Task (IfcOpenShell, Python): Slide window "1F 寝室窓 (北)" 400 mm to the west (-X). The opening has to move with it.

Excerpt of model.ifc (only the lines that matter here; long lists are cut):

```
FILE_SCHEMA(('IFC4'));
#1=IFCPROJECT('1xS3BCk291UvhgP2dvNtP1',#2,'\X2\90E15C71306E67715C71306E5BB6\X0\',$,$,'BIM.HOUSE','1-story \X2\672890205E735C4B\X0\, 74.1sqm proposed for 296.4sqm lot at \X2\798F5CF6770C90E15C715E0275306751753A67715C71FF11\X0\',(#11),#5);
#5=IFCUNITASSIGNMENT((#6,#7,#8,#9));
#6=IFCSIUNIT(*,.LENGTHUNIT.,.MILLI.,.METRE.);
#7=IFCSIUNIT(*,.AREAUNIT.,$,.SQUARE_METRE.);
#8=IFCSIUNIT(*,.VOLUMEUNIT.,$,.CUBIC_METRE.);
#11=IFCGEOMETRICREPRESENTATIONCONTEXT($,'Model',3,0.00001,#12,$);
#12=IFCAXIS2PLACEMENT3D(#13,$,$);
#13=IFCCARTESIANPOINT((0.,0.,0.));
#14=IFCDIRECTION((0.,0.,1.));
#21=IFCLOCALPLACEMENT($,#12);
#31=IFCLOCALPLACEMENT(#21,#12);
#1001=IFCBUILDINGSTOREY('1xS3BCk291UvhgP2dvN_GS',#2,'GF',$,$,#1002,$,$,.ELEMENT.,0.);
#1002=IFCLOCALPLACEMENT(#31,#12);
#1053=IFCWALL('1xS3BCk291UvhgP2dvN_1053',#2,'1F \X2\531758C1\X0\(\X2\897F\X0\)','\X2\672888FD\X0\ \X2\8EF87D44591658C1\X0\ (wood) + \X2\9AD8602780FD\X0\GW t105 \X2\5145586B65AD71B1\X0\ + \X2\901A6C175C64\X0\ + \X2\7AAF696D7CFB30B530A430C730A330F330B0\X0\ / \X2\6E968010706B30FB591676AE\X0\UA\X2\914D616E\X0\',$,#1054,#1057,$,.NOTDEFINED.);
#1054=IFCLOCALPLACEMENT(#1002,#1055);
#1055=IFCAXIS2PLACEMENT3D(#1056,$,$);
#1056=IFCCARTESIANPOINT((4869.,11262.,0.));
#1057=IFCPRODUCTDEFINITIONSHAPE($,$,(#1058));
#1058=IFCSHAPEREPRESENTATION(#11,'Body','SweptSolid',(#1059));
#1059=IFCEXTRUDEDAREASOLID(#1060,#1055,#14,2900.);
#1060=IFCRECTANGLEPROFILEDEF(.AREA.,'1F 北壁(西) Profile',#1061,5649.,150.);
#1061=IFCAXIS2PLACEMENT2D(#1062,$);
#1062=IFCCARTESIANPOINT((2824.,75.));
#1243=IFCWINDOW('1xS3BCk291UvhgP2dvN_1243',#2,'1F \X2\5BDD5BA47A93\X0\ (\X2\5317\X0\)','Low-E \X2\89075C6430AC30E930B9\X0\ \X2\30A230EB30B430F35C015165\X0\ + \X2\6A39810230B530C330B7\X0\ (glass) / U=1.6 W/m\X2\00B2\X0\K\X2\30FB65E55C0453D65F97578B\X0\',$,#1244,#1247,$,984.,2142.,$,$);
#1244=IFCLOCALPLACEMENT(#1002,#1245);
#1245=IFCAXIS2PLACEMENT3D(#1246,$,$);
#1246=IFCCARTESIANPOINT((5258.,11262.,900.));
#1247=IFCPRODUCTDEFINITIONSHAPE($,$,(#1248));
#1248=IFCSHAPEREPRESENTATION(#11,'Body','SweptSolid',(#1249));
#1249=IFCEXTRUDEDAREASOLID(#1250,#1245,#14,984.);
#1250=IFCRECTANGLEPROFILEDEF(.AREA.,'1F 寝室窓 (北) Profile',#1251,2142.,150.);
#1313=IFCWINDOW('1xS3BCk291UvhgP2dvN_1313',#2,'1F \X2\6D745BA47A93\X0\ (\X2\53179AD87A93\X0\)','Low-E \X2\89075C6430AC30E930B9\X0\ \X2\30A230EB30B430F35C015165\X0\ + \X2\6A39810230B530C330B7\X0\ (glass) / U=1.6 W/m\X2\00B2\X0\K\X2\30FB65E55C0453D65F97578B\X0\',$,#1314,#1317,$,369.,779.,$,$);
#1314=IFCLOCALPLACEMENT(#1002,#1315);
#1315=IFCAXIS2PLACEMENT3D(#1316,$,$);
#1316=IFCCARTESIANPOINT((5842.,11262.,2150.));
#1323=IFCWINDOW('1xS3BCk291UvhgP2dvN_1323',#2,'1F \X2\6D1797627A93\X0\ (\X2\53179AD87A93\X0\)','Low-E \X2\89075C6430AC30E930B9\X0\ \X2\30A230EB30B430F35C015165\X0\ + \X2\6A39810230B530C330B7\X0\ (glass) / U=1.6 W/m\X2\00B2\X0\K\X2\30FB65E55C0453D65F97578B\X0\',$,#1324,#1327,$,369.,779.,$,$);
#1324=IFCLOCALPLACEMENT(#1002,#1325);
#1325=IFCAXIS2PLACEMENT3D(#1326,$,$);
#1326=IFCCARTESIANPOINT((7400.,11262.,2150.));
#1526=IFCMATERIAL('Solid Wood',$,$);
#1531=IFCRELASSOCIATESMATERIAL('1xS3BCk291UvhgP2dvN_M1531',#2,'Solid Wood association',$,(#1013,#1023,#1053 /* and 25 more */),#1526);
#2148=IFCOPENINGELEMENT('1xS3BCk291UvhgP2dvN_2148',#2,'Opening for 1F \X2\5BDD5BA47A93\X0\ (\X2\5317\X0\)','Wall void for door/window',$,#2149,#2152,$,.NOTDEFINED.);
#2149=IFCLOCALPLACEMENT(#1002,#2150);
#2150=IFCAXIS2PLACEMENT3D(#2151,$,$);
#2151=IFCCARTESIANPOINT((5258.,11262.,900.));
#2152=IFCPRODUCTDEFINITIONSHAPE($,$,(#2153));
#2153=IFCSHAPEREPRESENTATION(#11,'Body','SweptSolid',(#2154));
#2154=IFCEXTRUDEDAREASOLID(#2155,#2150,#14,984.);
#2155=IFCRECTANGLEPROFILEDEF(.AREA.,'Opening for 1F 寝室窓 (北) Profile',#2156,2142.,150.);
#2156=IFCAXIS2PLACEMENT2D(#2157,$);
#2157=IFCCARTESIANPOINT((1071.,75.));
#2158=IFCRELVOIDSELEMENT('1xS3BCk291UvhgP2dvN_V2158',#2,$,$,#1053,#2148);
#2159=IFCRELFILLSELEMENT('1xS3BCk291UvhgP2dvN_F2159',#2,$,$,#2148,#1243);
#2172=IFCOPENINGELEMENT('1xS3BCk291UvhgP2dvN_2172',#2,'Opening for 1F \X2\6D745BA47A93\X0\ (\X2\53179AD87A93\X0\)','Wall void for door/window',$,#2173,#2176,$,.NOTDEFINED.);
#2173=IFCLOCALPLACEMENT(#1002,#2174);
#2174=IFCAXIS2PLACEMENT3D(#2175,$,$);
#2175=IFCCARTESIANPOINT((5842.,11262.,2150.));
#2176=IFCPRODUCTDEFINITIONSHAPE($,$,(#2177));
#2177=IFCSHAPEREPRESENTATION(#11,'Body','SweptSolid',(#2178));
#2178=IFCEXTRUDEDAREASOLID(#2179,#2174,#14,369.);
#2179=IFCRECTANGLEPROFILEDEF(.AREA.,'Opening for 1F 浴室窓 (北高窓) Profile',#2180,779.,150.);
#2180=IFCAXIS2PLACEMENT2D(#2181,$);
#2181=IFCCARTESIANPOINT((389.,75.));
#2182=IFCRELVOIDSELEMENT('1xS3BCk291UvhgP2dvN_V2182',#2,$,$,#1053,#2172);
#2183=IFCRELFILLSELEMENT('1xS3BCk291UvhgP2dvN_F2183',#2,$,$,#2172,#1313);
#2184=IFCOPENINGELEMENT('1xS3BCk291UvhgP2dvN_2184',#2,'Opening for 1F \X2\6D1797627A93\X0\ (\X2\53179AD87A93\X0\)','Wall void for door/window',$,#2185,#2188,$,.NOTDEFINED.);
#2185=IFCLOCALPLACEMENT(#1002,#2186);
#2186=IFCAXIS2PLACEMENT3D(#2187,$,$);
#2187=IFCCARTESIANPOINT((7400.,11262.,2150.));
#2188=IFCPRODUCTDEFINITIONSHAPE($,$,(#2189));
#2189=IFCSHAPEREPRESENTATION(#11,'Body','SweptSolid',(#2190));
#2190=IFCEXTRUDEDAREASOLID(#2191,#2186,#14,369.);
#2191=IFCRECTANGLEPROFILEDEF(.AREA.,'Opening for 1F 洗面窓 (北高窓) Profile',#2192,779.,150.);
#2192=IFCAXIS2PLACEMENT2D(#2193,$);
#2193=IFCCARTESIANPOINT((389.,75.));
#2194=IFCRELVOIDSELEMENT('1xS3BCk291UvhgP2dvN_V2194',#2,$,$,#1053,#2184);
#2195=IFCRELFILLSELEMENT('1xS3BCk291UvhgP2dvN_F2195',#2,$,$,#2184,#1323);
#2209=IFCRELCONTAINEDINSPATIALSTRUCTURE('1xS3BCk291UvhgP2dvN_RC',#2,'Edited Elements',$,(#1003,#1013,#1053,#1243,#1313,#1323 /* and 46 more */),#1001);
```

```python
import ifcopenshell
import ifcopenshell.api.geometry
import ifcopenshell.util.placement
import ifcopenshell.util.unit

model = ifcopenshell.open("model.ifc")
unit_scale = ifcopenshell.util.unit.calculate_unit_scale(model)

window = model.by_guid("1xS3BCk291UvhgP2dvN_1243")
opening = window.FillsVoids[0].RelatingOpeningElement
wall = opening.VoidsElements[0].RelatingBuildingElement

wall_matrix = ifcopenshell.util.placement.get_local_placement(wall.ObjectPlacement)
shift = wall_matrix[:3, 0] * -0.4 / unit_scale
before = ifcopenshell.util.placement.get_local_placement(window.ObjectPlacement)[:3, 3].copy()

# The window is not placed relative to its opening, so move both.
for product in (opening, window):
    matrix = ifcopenshell.util.placement.get_local_placement(product.ObjectPlacement)
    matrix[:3, 3] += shift
    ifcopenshell.api.geometry.edit_object_placement(model, product=product, matrix=matrix, is_si=False)

after = ifcopenshell.util.placement.get_local_placement(window.ObjectPlacement)[:3, 3]
print("window moved by", (after - before).round(3) + 0.0)

model.write("model_rev.ifc")
```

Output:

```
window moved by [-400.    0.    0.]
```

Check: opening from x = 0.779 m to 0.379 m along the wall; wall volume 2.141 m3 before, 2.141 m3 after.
